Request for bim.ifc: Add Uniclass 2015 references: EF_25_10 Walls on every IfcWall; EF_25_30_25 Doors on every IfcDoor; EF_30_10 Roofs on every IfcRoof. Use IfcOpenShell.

First a look at what the model holds.

```python
import ifcopenshell

model = ifcopenshell.open("bim.ifc")
print(model.schema)
print("classifications:", [c.Name for c in model.by_type("IfcClassification")])
for ifc_class in ("IfcDoor", "IfcRoof", "IfcStair", "IfcWall", "IfcWindow"):
    print(ifc_class, len(model.by_type(ifc_class)))
```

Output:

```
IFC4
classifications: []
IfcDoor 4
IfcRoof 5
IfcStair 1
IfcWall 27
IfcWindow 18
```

```python
import ifcopenshell
import ifcopenshell.api.classification

model = ifcopenshell.open("bim.ifc")

system = ifcopenshell.api.classification.add_classification(model, classification="Uniclass 2015")

codes = {
    "IfcWall": ("EF_25_10", "Walls"),
    "IfcDoor": ("EF_25_30_25", "Doors"),
    "IfcRoof": ("EF_30_10", "Roofs"),
}
for ifc_class, (code, name) in codes.items():
    products = model.by_type(ifc_class)
    ifcopenshell.api.classification.add_reference(
        model, products=products, classification=system, identification=code, name=name
    )
    print(code, len(products))

model.write("bim_updated.ifc")
```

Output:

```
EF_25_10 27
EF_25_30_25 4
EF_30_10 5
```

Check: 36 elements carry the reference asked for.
